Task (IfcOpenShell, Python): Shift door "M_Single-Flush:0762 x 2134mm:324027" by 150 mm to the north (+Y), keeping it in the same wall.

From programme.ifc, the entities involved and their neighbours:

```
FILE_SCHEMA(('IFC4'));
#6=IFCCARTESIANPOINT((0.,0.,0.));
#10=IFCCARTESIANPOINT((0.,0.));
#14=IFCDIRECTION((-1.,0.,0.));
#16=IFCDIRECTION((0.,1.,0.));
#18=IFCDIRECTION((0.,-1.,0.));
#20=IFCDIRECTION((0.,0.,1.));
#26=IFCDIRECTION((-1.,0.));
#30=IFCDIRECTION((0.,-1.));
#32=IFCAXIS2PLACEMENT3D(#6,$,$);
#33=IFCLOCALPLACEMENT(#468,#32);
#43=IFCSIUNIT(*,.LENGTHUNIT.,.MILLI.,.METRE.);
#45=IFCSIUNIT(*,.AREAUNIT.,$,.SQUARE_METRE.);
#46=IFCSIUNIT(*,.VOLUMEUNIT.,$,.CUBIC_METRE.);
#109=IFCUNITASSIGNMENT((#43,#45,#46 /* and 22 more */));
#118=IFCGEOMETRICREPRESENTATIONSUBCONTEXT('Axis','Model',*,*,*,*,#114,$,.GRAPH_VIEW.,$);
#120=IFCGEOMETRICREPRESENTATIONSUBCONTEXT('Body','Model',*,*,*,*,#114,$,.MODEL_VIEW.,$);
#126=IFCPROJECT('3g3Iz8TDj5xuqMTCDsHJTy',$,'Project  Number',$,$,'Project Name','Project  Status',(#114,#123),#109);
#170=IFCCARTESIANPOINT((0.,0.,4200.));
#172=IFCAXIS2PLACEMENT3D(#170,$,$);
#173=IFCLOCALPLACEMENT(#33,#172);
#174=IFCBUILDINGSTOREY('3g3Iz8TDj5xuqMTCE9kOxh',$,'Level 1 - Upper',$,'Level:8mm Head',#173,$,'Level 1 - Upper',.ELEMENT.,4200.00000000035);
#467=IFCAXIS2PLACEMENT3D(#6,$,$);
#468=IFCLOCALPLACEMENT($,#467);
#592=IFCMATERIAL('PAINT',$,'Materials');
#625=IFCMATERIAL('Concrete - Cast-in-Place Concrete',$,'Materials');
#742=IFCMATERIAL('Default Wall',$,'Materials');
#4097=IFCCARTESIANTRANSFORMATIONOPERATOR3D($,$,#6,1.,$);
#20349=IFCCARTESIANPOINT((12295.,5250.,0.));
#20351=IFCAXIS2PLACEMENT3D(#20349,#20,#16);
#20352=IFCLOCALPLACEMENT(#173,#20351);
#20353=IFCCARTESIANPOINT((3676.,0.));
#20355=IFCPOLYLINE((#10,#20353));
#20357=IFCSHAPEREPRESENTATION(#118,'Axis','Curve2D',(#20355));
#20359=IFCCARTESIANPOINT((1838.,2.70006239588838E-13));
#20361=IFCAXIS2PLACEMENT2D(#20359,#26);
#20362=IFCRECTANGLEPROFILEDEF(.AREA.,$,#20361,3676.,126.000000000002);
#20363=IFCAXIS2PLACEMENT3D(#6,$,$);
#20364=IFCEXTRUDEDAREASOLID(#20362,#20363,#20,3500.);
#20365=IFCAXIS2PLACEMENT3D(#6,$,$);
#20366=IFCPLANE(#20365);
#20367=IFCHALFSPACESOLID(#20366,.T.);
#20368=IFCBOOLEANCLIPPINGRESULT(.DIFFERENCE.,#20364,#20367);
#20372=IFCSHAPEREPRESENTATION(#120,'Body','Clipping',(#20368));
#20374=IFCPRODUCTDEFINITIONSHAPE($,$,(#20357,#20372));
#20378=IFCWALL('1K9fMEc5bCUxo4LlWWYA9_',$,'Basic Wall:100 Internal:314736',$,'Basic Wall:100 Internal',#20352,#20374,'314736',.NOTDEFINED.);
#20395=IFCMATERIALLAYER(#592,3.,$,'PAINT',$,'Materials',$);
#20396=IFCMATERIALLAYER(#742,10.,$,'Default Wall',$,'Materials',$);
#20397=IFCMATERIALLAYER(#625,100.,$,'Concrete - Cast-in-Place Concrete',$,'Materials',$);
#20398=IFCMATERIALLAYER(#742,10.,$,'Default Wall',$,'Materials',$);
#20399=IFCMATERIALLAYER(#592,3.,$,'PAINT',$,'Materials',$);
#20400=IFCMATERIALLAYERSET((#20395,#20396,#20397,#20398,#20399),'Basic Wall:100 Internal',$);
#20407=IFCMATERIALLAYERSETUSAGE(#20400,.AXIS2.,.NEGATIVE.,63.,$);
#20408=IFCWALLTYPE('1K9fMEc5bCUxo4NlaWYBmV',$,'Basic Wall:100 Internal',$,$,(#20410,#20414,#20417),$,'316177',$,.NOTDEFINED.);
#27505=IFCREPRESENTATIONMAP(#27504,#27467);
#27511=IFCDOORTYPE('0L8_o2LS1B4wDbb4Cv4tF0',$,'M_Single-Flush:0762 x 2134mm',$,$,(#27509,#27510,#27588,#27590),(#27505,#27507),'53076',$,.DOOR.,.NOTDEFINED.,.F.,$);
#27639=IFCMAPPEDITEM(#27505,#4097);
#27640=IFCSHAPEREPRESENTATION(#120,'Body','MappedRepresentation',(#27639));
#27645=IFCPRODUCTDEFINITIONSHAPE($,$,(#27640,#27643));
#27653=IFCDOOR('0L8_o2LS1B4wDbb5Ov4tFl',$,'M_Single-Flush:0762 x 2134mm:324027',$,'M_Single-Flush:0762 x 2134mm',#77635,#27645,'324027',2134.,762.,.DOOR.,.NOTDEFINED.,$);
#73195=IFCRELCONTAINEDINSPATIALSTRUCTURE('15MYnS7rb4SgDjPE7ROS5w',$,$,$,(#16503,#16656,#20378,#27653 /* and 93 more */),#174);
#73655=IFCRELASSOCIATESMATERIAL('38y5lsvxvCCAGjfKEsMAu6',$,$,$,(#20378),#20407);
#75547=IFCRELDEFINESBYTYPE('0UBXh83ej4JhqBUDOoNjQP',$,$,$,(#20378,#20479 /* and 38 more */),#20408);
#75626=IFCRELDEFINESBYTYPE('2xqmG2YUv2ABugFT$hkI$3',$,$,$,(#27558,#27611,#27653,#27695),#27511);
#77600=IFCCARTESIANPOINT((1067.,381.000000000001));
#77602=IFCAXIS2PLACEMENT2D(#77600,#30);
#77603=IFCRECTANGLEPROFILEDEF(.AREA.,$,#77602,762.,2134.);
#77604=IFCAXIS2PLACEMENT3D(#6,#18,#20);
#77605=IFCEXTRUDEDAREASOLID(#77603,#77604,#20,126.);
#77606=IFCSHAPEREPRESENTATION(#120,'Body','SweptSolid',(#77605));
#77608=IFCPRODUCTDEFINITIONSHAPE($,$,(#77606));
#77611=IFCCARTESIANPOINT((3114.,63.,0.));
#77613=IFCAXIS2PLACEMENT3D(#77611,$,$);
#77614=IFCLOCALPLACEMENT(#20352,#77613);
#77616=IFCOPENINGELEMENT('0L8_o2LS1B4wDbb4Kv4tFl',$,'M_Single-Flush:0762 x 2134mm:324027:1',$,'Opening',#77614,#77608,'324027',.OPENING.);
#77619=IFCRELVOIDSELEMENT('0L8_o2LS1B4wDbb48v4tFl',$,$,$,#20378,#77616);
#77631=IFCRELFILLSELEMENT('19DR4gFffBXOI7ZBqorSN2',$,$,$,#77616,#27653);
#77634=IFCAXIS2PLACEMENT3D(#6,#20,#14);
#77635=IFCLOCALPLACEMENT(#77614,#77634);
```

```python
import ifcopenshell
import ifcopenshell.api.geometry
import ifcopenshell.util.placement

model = ifcopenshell.open("programme.ifc")

door = model.by_guid("0L8_o2LS1B4wDbb5Ov4tFl")
opening = door.FillsVoids[0].RelatingOpeningElement
wall = opening.VoidsElements[0].RelatingBuildingElement

wall_matrix = ifcopenshell.util.placement.get_local_placement(wall.ObjectPlacement)
shift = wall_matrix[:3, 0] * 150.0
before = ifcopenshell.util.placement.get_local_placement(door.ObjectPlacement)[:3, 3].copy()

# The door is placed relative to its opening, so it follows when the opening moves.
matrix = ifcopenshell.util.placement.get_local_placement(opening.ObjectPlacement)
matrix[:3, 3] += shift
ifcopenshell.api.geometry.edit_object_placement(
    model, product=opening, matrix=matrix, is_si=False, should_transform_children=True
)

after = ifcopenshell.util.placement.get_local_placement(door.ObjectPlacement)[:3, 3]
print("door moved by", (after - before).round(3) + 0.0)

model.write("programme_edited.ifc")
```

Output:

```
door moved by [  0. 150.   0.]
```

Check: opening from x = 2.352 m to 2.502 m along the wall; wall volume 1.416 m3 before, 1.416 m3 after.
